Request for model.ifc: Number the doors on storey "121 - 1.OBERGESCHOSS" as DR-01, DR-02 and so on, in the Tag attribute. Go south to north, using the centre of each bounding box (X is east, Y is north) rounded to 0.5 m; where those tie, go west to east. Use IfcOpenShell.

First a look at what the model holds.

```python
import ifcopenshell
import ifcopenshell.util.element
import ifcopenshell.util.placement

model = ifcopenshell.open("model.ifc")
print(model.schema)
storey = next(s for s in model.by_type("IfcBuildingStorey") if s.Name == "121 - 1.OBERGESCHOSS")
doors = [e for e in ifcopenshell.util.element.get_decomposition(storey) if e.is_a("IfcDoor")]
for e in sorted(doors, key=lambda e: e.id()):
    origin = ifcopenshell.util.placement.get_local_placement(e.ObjectPlacement)[:3, 3]
    print(e.id(), e.Tag, e.Name, origin.round(2) + 0.0, sep=" | ")
```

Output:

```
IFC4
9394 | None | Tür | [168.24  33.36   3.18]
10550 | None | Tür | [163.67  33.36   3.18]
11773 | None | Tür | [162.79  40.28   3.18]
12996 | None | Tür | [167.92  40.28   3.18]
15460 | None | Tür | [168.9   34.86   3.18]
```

```python
import ifcopenshell
import ifcopenshell.geom
import ifcopenshell.util.element
import ifcopenshell.util.shape

model = ifcopenshell.open("model.ifc")
settings = ifcopenshell.geom.settings()
settings.set("use-world-coords", True)


def centre(element):
    shape = ifcopenshell.geom.create_shape(settings, element)
    return ifcopenshell.util.shape.get_bbox_centroid(shape.geometry)


storey = next(s for s in model.by_type("IfcBuildingStorey") if s.Name == "121 - 1.OBERGESCHOSS")
doors = [e for e in ifcopenshell.util.element.get_decomposition(storey) if e.is_a("IfcDoor")]

# Insertion points can sit at a corner or the storey origin, so sort by the geometry (in metres).
centres = {e: centre(e) for e in doors}
doors.sort(key=lambda e: (round(centres[e][1] / 0.5), centres[e][0]))

for i, e in enumerate(doors, start=1):
    number = f"DR-{i:02d}"
    e.Tag = number
    print(e.id(), number)

model.write("model_rev.ifc")
```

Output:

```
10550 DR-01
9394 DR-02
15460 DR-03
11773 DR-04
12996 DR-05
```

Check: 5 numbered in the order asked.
